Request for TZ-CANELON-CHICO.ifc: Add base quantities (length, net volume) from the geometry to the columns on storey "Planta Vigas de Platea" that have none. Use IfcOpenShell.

First a look at what the model holds.

```python
import ifcopenshell
import ifcopenshell.util.element
import ifcopenshell.util.unit

model = ifcopenshell.open("TZ-CANELON-CHICO.ifc")
print(model.schema)
for unit_type in ("LENGTHUNIT", "AREAUNIT", "VOLUMEUNIT"):
    print(unit_type, ifcopenshell.util.unit.calculate_unit_scale(model, unit_type))
storey = next(s for s in model.by_type("IfcBuildingStorey") if s.Name == "Planta Vigas de Platea")
columns = [e for e in ifcopenshell.util.element.get_decomposition(storey) if e.is_a("IfcColumn")]
for e in sorted(columns, key=lambda e: e.id()):
    print(e.id(), e.is_a(), e.Name, list(ifcopenshell.util.element.get_psets(e, qtos_only=True)), sep=" | ")
```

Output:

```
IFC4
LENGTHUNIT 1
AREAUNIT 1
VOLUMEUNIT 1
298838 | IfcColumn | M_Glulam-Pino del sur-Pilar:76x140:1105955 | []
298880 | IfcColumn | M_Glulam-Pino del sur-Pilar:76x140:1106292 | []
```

```python
import ifcopenshell
import ifcopenshell.api.pset
import ifcopenshell.geom
import ifcopenshell.util.element
import ifcopenshell.util.shape
import ifcopenshell.util.unit

model = ifcopenshell.open("TZ-CANELON-CHICO.ifc")
unit_scale = ifcopenshell.util.unit.calculate_unit_scale(model)
volume_scale = ifcopenshell.util.unit.calculate_unit_scale(model, "VOLUMEUNIT")
settings = ifcopenshell.geom.settings()

storey = next(s for s in model.by_type("IfcBuildingStorey") if s.Name == "Planta Vigas de Platea")
columns = [e for e in ifcopenshell.util.element.get_decomposition(storey) if e.is_a("IfcColumn")]

for e in sorted(columns, key=lambda e: e.id()):
    if ifcopenshell.util.element.get_psets(e, qtos_only=True, should_inherit=False):
        continue
    # Geometry comes back in metres, in the element's own axes.
    shape = ifcopenshell.geom.create_shape(settings, e)
    values = {
        "Length": ifcopenshell.util.shape.get_z(shape.geometry) / unit_scale,
        "NetVolume": ifcopenshell.util.shape.get_volume(shape.geometry) / volume_scale,
    }
    qto = ifcopenshell.api.pset.add_qto(model, product=e, name="Qto_ColumnBaseQuantities")
    ifcopenshell.api.pset.edit_qto(model, qto=qto, properties=values)
    print(e.id(), {k: round(v, 3) for k, v in values.items()})

model.write("TZ-CANELON-CHICO_v2.ifc")
```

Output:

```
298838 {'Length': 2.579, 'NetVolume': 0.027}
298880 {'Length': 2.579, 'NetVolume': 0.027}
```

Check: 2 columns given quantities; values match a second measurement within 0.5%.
